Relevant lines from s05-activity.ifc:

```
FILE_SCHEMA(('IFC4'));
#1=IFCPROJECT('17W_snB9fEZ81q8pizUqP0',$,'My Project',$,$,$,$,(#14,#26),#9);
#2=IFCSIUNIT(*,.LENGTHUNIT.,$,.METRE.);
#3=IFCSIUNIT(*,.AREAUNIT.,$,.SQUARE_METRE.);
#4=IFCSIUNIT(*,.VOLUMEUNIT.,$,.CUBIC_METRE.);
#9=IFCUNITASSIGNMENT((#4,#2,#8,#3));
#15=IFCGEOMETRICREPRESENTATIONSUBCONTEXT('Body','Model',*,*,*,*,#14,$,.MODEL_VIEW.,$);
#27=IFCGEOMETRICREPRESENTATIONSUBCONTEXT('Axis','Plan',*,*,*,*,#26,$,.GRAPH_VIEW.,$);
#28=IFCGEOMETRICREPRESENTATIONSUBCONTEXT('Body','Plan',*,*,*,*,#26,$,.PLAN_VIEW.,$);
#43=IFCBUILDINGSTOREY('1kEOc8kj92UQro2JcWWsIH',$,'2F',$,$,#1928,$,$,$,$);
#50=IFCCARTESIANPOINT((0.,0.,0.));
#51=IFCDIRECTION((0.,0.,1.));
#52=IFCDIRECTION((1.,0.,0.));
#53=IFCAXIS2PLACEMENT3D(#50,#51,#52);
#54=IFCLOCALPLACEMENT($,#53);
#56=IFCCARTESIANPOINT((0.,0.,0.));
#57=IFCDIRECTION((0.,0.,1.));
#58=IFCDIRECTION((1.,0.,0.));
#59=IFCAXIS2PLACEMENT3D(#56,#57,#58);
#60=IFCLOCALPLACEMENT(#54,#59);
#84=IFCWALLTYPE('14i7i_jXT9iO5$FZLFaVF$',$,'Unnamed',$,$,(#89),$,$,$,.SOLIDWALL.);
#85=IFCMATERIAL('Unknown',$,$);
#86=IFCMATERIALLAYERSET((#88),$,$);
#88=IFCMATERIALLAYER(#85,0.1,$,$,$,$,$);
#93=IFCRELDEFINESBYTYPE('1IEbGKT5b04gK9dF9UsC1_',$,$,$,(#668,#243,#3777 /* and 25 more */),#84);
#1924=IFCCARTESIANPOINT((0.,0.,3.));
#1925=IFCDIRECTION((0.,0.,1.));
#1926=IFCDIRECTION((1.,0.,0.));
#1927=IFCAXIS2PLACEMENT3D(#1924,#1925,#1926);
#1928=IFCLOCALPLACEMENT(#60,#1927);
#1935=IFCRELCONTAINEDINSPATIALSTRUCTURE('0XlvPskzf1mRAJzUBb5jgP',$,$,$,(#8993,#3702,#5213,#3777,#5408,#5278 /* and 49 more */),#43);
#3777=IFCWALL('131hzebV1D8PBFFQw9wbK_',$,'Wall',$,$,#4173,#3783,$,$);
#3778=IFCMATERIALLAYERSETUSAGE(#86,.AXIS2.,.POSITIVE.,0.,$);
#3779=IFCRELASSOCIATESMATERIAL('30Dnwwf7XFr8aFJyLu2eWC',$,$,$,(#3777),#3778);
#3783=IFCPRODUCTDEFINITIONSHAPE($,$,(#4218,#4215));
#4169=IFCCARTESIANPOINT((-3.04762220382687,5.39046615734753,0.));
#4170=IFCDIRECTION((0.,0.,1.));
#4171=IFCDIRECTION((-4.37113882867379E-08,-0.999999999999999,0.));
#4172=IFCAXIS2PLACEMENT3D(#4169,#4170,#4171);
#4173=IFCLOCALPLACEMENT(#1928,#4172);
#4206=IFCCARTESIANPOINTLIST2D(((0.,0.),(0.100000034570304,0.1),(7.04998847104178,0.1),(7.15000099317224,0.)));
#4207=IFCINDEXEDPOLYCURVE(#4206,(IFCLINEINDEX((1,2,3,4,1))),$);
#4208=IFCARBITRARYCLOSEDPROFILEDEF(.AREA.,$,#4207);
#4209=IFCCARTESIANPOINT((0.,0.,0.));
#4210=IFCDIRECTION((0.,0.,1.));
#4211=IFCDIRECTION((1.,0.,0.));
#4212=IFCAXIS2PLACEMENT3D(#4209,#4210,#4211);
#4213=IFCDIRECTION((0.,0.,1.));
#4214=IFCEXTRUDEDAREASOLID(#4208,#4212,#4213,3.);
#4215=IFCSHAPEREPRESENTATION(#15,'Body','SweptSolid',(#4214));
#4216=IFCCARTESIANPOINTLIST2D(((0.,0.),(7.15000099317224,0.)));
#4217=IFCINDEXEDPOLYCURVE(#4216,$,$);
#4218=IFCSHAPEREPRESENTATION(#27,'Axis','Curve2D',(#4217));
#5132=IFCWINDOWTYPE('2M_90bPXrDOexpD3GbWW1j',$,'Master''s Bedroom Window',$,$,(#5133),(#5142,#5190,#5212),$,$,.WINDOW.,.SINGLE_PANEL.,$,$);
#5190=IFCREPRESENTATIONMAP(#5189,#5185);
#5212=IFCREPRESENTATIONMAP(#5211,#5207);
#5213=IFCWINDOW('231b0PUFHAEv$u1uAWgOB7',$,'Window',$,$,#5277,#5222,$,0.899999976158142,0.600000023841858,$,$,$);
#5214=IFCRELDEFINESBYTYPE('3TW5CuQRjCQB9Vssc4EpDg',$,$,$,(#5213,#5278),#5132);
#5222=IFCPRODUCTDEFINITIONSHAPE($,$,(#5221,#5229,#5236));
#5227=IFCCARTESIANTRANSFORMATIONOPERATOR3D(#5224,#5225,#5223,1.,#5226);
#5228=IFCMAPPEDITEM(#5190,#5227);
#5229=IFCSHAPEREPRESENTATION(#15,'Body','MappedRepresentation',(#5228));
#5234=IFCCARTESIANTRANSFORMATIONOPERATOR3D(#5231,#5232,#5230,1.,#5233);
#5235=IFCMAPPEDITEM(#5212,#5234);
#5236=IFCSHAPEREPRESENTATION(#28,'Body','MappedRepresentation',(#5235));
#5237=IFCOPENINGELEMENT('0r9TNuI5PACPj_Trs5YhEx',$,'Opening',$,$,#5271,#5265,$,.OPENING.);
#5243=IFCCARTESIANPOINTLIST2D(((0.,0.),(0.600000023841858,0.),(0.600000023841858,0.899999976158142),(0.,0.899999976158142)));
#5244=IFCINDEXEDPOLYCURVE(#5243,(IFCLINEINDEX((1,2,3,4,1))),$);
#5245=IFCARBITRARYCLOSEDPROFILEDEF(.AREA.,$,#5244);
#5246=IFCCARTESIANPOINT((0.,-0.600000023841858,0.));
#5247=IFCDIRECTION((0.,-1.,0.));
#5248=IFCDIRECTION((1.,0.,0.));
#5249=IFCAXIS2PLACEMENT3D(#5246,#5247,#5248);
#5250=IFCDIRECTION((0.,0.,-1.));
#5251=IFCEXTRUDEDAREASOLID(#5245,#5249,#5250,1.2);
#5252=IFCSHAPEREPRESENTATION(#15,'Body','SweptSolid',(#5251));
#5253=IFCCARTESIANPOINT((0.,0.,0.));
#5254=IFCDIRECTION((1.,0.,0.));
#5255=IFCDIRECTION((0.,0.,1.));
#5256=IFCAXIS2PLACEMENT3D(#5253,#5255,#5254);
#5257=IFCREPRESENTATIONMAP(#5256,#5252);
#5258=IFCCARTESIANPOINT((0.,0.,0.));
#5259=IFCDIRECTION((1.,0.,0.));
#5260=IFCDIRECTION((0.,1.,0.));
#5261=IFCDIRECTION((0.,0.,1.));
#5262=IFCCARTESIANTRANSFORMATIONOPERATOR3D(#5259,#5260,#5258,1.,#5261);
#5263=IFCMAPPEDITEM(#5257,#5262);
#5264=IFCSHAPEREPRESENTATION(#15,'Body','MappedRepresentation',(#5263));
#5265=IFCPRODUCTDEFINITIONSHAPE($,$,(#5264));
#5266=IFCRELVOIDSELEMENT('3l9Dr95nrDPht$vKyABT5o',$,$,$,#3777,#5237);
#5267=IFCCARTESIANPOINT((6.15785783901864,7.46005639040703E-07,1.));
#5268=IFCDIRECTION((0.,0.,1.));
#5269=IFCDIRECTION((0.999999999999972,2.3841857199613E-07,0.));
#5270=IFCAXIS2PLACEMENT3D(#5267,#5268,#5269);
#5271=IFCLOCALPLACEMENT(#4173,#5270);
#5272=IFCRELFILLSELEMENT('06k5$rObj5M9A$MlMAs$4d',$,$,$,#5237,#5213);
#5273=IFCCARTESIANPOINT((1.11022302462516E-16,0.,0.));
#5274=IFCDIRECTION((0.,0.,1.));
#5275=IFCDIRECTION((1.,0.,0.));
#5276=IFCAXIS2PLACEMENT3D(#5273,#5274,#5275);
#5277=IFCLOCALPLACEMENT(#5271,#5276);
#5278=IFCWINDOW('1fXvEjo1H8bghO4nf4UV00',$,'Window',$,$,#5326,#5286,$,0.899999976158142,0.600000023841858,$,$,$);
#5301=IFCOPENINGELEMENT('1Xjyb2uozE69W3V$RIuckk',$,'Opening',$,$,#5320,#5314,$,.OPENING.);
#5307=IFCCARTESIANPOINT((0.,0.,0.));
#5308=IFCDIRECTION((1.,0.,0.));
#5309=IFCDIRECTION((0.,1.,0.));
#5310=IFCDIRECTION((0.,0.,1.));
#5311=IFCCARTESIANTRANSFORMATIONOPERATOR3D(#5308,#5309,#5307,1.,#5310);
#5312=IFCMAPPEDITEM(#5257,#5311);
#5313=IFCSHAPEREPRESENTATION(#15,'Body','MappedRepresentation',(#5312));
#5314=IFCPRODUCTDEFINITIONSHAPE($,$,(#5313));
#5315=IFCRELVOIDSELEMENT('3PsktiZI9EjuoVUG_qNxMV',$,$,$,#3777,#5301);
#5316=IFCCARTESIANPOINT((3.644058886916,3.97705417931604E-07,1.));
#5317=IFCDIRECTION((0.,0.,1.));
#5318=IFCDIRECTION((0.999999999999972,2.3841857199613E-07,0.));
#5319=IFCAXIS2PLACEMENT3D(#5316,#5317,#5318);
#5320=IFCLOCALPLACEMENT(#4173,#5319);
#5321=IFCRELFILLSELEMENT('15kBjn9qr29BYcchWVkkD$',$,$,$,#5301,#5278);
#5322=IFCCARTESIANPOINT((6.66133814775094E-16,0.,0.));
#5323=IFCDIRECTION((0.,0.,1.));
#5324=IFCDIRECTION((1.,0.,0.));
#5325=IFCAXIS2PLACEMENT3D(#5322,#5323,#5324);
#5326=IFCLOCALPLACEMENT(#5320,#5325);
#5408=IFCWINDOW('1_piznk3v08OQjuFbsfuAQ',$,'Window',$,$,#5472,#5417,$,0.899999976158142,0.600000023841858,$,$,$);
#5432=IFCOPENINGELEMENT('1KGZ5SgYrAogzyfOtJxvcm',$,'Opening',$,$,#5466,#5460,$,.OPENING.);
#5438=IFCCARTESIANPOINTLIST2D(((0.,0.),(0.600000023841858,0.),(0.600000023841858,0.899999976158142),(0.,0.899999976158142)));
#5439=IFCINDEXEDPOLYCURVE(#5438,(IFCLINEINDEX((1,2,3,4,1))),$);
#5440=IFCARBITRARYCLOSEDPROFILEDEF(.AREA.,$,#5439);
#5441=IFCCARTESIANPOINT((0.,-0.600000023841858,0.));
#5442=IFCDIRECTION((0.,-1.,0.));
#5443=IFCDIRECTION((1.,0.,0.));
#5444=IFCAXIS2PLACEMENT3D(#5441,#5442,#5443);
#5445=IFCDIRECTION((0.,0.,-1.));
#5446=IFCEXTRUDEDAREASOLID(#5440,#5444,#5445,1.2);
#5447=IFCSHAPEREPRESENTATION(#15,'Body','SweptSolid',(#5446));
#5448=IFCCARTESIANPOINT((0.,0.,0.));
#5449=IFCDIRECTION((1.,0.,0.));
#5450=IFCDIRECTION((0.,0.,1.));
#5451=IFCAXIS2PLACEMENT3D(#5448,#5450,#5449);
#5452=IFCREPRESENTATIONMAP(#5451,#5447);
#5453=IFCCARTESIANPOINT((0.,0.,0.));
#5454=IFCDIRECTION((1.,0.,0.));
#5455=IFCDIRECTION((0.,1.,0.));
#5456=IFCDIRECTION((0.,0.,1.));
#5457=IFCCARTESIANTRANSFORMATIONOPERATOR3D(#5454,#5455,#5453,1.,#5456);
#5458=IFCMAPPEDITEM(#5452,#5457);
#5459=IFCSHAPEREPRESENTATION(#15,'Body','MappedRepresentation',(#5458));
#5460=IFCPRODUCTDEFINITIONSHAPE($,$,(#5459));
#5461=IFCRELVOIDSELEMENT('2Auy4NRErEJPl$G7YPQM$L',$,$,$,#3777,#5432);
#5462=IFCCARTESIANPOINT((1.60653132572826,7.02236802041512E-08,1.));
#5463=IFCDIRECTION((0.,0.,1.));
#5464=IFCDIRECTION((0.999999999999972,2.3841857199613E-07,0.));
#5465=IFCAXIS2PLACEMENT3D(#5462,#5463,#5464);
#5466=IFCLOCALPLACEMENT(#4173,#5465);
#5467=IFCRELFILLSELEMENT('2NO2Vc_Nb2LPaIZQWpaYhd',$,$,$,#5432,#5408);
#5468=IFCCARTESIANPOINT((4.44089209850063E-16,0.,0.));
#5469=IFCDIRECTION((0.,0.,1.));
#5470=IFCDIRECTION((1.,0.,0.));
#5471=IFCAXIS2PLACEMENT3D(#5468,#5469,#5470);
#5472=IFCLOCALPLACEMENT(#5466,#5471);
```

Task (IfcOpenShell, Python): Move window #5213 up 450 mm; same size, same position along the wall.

```python
import numpy as np
import ifcopenshell
import ifcopenshell.api.geometry
import ifcopenshell.util.placement
import ifcopenshell.util.unit

model = ifcopenshell.open("s05-activity.ifc")
unit_scale = ifcopenshell.util.unit.calculate_unit_scale(model)

window = model.by_guid("231b0PUFHAEv$u1uAWgOB7")
opening = window.FillsVoids[0].RelatingOpeningElement
dz = 0.45

shift = np.array([0.0, 0.0, dz])
# The window is placed relative to its opening, so it follows when the opening moves.
matrix = ifcopenshell.util.placement.get_local_placement(opening.ObjectPlacement)
matrix[:3, 3] += shift
ifcopenshell.api.geometry.edit_object_placement(
    model, product=opening, matrix=matrix, is_si=False, should_transform_children=True
)

print(f"moved by {dz * unit_scale:+.3f} m")

model.write("s05-activity-out.ifc")
```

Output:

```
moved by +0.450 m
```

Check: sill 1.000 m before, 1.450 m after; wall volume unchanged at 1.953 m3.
